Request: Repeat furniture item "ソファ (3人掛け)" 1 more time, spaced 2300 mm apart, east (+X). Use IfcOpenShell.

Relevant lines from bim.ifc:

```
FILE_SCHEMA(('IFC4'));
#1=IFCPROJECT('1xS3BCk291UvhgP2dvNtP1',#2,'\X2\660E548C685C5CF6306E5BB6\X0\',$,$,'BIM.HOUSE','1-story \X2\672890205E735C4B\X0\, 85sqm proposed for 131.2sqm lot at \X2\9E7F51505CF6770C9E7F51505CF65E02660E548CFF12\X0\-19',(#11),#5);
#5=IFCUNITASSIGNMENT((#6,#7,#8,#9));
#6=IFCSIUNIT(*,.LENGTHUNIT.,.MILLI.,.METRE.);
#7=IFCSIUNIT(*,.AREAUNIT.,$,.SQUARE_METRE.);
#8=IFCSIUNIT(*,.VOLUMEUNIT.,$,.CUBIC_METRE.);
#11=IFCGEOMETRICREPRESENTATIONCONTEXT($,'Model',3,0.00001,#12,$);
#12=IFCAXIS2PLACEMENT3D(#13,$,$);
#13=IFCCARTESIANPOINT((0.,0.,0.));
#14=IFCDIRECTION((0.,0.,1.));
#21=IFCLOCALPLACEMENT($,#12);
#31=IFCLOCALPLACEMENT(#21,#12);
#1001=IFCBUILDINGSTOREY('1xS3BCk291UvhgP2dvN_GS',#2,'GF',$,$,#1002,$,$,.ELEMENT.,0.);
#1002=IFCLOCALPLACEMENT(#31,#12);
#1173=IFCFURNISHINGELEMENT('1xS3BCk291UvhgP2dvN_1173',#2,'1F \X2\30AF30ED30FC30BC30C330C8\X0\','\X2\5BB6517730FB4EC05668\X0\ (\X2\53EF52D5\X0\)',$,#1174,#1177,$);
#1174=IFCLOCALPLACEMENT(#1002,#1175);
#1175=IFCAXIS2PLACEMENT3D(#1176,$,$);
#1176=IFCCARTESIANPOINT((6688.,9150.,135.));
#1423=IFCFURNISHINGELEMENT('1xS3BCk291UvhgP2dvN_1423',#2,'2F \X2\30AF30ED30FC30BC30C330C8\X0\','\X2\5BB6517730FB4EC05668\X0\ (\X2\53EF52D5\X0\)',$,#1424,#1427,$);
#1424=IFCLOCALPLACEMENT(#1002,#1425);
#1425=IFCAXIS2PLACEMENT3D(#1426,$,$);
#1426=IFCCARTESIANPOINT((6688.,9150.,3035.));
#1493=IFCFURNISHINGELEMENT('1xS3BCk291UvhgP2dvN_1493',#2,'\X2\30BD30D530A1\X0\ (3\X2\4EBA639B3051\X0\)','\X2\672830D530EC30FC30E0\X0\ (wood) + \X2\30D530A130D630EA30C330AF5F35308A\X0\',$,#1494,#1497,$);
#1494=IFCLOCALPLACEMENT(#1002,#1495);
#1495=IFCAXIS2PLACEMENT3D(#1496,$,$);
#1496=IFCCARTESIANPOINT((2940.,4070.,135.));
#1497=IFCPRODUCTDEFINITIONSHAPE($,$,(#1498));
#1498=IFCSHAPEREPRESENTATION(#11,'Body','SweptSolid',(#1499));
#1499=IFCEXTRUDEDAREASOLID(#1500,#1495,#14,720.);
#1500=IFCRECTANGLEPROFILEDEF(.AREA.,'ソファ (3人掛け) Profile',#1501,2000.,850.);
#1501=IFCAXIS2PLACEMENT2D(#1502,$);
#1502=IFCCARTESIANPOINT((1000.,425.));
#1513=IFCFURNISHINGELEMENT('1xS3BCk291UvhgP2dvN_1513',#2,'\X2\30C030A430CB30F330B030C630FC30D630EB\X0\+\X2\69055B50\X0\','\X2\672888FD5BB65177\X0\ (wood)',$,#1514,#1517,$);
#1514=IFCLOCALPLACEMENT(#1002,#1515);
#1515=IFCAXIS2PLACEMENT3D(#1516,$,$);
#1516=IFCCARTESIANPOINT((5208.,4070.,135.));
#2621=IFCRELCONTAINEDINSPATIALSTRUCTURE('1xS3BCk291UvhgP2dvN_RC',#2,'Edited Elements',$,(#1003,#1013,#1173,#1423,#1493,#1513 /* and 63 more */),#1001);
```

```python
import numpy as np
import ifcopenshell
import ifcopenshell.api.geometry
import ifcopenshell.api.root
import ifcopenshell.util.element
import ifcopenshell.util.placement

model = ifcopenshell.open("bim.ifc")


def reuse_history(source, copy):
    """copy_class also copies each property set's owner history, people and application; keep the originals."""
    for rel in copy.IsDefinedBy:
        if rel.is_a("IfcRelDefinesByProperties") and (history := rel.RelatingPropertyDefinition.OwnerHistory):
            rel.RelatingPropertyDefinition.OwnerHistory = source.OwnerHistory
            ifcopenshell.util.element.remove_deep2(model, history)


source = model.by_id(1493)
base = ifcopenshell.util.placement.get_local_placement(source.ObjectPlacement)
step = np.array([1.0, 0.0, 0.0]) * 2300.0

for i in range(1, 2):
    copy = ifcopenshell.api.root.copy_class(model, product=source)
    copy.Representation = ifcopenshell.util.element.copy_deep(
        model, source.Representation, exclude=["IfcGeometricRepresentationContext", "IfcRepresentationMap"]
    )
    reuse_history(source, copy)
    matrix = base.copy()
    matrix[:3, 3] += i * step
    print("added at", matrix[:3, 3].round(3) + 0.0)
    ifcopenshell.api.geometry.edit_object_placement(model, product=copy, matrix=matrix, is_si=False)

model.write("bim_v2.ifc")
```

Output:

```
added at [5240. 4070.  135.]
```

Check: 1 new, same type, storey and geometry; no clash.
